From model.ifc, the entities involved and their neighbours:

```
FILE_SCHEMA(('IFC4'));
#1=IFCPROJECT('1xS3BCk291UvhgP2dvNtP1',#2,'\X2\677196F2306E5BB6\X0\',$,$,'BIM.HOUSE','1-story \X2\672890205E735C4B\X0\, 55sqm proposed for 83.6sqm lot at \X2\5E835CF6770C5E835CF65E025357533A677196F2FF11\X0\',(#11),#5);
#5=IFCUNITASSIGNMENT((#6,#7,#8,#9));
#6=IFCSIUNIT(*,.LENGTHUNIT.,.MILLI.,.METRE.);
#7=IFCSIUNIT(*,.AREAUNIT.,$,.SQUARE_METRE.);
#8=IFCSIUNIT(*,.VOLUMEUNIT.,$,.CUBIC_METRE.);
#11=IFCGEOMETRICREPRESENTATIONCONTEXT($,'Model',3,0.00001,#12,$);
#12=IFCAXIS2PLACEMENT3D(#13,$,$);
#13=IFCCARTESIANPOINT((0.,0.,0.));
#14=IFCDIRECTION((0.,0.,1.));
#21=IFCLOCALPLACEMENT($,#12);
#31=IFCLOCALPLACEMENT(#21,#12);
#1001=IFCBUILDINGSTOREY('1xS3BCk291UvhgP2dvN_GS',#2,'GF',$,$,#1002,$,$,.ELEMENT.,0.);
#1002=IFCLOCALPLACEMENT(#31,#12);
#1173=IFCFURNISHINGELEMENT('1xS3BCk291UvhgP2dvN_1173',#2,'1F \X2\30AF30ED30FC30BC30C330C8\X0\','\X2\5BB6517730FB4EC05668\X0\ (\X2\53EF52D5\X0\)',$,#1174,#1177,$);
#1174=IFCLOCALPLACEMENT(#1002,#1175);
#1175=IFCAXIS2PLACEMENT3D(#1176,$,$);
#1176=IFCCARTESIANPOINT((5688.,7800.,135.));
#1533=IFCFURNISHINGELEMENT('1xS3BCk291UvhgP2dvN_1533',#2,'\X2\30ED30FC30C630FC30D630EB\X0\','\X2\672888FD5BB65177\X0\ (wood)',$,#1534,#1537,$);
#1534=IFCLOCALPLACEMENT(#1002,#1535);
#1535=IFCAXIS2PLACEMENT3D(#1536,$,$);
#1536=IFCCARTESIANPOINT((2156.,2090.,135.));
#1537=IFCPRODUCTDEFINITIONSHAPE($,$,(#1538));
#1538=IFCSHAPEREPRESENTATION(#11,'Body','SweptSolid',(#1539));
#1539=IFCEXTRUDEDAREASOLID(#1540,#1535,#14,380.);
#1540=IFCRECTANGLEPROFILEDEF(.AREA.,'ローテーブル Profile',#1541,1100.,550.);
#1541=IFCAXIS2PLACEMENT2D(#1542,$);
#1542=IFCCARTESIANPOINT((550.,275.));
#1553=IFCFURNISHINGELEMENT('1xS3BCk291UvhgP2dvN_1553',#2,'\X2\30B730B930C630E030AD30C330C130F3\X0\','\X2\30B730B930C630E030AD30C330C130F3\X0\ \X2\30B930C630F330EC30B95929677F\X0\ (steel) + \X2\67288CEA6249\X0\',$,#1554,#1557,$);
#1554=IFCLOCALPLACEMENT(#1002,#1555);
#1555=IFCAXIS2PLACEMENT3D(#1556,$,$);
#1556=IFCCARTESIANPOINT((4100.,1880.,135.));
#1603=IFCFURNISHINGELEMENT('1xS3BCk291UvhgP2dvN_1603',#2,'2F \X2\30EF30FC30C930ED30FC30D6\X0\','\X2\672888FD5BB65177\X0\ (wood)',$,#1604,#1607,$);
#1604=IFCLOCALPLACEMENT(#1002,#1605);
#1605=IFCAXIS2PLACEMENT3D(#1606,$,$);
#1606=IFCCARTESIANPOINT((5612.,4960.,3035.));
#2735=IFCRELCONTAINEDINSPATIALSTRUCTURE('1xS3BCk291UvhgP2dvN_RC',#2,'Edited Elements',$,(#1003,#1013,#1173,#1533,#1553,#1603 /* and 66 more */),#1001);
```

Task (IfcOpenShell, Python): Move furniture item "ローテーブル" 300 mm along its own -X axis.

```python
import ifcopenshell
import ifcopenshell.api.geometry
import ifcopenshell.util.placement
import ifcopenshell.util.unit

model = ifcopenshell.open("model.ifc")
unit_scale = ifcopenshell.util.unit.calculate_unit_scale(model)

item = model.by_guid("1xS3BCk291UvhgP2dvN_1533")
matrix = ifcopenshell.util.placement.get_local_placement(item.ObjectPlacement)
matrix[:3, 3] -= matrix[:3, 0] * 0.3 / unit_scale
ifcopenshell.api.geometry.edit_object_placement(model, product=item, matrix=matrix, is_si=False)

print(ifcopenshell.util.placement.get_local_placement(item.ObjectPlacement).round(3) + 0.0)

model.write("model_edited.ifc")
```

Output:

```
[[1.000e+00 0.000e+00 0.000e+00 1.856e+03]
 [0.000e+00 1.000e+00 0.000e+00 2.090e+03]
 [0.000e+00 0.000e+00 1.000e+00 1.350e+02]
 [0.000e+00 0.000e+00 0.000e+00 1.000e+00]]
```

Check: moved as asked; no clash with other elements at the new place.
